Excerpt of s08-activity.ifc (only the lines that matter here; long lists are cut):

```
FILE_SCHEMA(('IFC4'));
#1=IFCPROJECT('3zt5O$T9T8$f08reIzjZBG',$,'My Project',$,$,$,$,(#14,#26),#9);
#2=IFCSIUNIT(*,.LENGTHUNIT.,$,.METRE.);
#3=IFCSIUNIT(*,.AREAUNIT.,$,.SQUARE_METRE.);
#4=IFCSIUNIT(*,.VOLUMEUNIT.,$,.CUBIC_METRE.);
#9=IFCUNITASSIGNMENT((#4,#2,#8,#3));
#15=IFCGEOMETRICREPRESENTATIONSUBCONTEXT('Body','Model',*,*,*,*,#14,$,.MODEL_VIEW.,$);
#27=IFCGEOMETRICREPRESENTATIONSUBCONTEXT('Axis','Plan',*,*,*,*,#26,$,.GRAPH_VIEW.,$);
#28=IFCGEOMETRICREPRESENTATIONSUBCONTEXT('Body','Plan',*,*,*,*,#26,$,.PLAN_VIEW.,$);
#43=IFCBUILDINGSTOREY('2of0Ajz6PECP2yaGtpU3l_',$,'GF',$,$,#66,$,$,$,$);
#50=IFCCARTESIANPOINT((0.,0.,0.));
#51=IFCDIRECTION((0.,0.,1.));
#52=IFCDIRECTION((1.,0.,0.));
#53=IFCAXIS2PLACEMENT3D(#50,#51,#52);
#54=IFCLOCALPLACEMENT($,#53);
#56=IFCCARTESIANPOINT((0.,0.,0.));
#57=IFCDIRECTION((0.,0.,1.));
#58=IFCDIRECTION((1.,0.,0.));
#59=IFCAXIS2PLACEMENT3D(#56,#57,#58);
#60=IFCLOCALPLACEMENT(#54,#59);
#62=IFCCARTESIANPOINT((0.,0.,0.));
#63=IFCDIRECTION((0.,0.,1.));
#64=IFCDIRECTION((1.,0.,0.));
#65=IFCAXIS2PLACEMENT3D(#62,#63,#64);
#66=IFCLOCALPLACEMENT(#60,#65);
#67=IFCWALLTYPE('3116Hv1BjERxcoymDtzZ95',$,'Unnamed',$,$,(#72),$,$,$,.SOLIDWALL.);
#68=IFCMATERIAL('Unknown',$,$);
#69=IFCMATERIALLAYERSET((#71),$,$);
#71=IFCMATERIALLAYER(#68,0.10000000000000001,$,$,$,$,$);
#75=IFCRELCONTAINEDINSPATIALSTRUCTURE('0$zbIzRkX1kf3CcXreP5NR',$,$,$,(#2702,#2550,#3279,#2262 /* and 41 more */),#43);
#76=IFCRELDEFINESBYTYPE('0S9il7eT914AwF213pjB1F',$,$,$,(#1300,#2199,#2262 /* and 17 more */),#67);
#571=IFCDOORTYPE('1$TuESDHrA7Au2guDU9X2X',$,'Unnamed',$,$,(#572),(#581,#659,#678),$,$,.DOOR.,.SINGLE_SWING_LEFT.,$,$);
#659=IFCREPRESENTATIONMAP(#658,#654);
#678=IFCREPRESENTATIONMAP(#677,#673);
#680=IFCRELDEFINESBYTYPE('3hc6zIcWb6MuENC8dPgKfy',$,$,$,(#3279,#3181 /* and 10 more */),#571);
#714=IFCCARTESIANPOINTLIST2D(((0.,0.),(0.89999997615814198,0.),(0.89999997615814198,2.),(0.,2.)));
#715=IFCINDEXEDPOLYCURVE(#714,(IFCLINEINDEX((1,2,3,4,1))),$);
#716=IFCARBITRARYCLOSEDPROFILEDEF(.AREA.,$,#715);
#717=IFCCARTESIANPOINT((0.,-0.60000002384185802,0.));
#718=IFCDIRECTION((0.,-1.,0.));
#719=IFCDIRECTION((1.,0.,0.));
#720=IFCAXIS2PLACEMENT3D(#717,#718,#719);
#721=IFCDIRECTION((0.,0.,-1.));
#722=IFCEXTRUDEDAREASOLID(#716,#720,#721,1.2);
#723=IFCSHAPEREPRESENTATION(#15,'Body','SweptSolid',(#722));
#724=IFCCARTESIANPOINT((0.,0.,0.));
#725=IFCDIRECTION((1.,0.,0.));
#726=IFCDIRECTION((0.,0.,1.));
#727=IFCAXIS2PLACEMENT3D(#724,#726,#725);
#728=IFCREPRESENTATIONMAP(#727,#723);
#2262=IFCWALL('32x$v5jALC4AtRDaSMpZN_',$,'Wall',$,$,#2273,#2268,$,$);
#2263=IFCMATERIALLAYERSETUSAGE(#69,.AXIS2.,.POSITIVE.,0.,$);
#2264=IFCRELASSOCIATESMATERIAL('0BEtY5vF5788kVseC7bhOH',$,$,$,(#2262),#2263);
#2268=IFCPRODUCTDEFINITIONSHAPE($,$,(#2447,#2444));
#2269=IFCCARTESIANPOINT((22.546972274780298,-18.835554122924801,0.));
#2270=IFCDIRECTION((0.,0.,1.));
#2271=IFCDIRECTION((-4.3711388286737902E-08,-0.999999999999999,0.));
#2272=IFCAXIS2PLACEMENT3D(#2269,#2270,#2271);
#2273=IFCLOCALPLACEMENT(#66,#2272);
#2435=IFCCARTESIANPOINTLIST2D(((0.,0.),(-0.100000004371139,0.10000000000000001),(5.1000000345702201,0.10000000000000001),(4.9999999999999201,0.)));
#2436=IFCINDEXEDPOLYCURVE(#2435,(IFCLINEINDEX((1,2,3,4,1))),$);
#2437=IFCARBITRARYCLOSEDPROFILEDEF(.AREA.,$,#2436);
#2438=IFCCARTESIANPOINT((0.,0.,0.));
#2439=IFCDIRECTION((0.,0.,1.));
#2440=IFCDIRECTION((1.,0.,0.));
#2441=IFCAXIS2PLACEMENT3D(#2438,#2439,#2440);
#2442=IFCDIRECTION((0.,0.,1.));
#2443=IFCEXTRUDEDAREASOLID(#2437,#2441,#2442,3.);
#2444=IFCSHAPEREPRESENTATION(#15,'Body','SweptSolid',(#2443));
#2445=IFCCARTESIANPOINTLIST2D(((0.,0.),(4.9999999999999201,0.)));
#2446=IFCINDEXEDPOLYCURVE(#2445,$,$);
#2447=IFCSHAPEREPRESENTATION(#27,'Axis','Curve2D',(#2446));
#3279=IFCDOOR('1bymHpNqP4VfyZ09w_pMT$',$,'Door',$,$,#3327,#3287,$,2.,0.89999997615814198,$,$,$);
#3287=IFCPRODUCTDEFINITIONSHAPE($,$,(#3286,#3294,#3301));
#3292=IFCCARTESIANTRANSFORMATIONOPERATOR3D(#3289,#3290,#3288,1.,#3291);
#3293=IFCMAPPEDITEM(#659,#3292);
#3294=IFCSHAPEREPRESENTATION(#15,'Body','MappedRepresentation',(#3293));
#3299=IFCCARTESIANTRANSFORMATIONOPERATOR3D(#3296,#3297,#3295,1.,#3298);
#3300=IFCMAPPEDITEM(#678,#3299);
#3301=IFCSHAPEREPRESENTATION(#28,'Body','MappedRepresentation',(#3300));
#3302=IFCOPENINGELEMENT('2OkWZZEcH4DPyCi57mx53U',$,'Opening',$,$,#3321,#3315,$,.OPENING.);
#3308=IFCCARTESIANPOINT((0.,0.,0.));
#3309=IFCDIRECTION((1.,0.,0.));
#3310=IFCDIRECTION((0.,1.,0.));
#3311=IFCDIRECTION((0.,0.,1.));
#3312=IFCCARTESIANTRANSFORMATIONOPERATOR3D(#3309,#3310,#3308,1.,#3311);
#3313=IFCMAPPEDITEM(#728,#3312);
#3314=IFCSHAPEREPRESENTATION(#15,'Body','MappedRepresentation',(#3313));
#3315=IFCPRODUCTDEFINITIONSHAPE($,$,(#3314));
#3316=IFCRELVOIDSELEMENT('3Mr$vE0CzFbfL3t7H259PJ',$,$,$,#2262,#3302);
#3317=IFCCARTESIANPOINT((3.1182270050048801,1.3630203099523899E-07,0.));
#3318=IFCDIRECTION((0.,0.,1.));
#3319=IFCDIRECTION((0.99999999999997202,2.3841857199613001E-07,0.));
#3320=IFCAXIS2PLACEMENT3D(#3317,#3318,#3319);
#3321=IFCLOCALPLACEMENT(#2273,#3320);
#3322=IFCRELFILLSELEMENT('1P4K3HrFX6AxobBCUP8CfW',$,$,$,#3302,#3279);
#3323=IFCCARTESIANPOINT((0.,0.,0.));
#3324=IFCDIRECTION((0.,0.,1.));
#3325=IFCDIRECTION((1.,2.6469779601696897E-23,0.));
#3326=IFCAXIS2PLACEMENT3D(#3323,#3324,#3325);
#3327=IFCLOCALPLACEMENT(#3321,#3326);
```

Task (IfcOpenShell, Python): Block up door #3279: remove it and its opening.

```python
import ifcopenshell
import ifcopenshell.api.feature
import ifcopenshell.api.root
import ifcopenshell.geom
import ifcopenshell.util.shape

model = ifcopenshell.open("s08-activity.ifc")
settings = ifcopenshell.geom.settings()


def volume(element):
    """Net volume in cubic metres, openings subtracted."""
    shape = ifcopenshell.geom.create_shape(settings, element)
    return ifcopenshell.util.shape.get_volume(shape.geometry)


door = model.by_id(3279)
opening = door.FillsVoids[0].RelatingOpeningElement
wall = opening.VoidsElements[0].RelatingBuildingElement
before = volume(wall)

ifcopenshell.api.root.remove_product(model, product=door)
ifcopenshell.api.feature.remove_feature(model, feature=opening)

after = volume(wall)

print(f"wall volume {before:.3f} -> {after:.3f} m3")

model.write("s08-activity_updated.ifc")
```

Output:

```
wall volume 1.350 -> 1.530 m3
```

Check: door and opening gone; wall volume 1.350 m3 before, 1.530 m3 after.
